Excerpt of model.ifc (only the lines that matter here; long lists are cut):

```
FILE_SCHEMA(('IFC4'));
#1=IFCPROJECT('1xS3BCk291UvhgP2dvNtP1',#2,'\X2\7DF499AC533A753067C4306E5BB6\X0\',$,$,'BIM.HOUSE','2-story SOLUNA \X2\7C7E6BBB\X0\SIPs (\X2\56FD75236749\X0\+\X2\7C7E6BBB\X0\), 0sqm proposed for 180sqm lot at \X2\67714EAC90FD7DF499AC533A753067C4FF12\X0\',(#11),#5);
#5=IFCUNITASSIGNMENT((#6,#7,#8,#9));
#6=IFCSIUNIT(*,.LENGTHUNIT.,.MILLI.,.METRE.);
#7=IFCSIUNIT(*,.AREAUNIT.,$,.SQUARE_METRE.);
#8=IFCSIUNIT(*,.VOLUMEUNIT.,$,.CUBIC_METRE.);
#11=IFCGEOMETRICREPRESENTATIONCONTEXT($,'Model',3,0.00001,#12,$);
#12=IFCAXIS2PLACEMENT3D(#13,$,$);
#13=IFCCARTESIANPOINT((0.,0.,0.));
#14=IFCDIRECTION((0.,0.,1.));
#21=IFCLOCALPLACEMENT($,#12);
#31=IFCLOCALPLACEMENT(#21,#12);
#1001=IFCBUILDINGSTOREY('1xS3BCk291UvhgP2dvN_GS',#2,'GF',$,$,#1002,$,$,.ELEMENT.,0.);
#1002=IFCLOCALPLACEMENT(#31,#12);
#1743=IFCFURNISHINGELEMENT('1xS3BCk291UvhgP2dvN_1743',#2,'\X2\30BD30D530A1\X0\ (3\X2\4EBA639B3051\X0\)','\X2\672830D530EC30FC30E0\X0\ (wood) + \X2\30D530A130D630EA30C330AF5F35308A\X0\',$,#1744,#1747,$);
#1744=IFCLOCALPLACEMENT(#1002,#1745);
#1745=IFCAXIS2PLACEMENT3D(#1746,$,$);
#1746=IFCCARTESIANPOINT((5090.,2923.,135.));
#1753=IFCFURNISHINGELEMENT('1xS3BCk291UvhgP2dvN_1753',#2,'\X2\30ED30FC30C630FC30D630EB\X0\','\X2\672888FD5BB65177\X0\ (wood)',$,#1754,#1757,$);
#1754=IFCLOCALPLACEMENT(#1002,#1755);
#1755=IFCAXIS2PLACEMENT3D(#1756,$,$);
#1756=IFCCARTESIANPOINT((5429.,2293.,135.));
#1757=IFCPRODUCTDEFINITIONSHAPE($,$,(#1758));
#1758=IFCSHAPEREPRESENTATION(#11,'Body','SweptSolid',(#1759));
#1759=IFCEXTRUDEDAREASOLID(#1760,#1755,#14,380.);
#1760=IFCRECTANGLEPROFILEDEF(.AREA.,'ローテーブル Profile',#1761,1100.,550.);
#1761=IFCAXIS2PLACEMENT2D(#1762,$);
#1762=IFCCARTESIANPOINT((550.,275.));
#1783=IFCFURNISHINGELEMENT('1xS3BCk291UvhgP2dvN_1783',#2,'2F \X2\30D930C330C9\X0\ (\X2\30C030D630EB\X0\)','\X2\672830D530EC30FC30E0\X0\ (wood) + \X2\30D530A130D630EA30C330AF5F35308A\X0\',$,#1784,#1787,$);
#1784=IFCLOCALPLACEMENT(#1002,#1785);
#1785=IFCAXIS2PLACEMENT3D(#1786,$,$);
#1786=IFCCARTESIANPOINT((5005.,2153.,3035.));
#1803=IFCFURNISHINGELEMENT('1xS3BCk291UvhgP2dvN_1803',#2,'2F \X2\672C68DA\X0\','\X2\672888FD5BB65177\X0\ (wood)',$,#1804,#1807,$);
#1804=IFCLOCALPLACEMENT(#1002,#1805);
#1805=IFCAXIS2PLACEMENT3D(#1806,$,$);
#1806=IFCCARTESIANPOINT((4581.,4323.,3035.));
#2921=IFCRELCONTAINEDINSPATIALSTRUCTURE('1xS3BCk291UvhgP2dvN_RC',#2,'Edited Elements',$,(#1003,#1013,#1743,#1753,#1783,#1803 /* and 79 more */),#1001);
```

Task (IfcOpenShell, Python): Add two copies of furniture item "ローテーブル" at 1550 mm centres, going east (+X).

```python
import numpy as np
import ifcopenshell
import ifcopenshell.api.geometry
import ifcopenshell.api.root
import ifcopenshell.util.element
import ifcopenshell.util.placement
import ifcopenshell.util.unit

model = ifcopenshell.open("model.ifc")
unit_scale = ifcopenshell.util.unit.calculate_unit_scale(model)


def reuse_history(source, copy):
    """copy_class also copies each property set's owner history, people and application; keep the originals."""
    for rel in copy.IsDefinedBy:
        if rel.is_a("IfcRelDefinesByProperties") and (history := rel.RelatingPropertyDefinition.OwnerHistory):
            rel.RelatingPropertyDefinition.OwnerHistory = source.OwnerHistory
            ifcopenshell.util.element.remove_deep2(model, history)


source = model.by_guid("1xS3BCk291UvhgP2dvN_1753")
base = ifcopenshell.util.placement.get_local_placement(source.ObjectPlacement)
step = np.array([1.0, 0.0, 0.0]) * 1.55 / unit_scale

for i in range(1, 3):
    copy = ifcopenshell.api.root.copy_class(model, product=source)
    copy.Representation = ifcopenshell.util.element.copy_deep(
        model, source.Representation, exclude=["IfcGeometricRepresentationContext", "IfcRepresentationMap"]
    )
    reuse_history(source, copy)
    matrix = base.copy()
    matrix[:3, 3] += i * step
    print("added at", matrix[:3, 3].round(3) + 0.0)
    ifcopenshell.api.geometry.edit_object_placement(model, product=copy, matrix=matrix, is_si=False)

model.write("model_v2.ifc")
```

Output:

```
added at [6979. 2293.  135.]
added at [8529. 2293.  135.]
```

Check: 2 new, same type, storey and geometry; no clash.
